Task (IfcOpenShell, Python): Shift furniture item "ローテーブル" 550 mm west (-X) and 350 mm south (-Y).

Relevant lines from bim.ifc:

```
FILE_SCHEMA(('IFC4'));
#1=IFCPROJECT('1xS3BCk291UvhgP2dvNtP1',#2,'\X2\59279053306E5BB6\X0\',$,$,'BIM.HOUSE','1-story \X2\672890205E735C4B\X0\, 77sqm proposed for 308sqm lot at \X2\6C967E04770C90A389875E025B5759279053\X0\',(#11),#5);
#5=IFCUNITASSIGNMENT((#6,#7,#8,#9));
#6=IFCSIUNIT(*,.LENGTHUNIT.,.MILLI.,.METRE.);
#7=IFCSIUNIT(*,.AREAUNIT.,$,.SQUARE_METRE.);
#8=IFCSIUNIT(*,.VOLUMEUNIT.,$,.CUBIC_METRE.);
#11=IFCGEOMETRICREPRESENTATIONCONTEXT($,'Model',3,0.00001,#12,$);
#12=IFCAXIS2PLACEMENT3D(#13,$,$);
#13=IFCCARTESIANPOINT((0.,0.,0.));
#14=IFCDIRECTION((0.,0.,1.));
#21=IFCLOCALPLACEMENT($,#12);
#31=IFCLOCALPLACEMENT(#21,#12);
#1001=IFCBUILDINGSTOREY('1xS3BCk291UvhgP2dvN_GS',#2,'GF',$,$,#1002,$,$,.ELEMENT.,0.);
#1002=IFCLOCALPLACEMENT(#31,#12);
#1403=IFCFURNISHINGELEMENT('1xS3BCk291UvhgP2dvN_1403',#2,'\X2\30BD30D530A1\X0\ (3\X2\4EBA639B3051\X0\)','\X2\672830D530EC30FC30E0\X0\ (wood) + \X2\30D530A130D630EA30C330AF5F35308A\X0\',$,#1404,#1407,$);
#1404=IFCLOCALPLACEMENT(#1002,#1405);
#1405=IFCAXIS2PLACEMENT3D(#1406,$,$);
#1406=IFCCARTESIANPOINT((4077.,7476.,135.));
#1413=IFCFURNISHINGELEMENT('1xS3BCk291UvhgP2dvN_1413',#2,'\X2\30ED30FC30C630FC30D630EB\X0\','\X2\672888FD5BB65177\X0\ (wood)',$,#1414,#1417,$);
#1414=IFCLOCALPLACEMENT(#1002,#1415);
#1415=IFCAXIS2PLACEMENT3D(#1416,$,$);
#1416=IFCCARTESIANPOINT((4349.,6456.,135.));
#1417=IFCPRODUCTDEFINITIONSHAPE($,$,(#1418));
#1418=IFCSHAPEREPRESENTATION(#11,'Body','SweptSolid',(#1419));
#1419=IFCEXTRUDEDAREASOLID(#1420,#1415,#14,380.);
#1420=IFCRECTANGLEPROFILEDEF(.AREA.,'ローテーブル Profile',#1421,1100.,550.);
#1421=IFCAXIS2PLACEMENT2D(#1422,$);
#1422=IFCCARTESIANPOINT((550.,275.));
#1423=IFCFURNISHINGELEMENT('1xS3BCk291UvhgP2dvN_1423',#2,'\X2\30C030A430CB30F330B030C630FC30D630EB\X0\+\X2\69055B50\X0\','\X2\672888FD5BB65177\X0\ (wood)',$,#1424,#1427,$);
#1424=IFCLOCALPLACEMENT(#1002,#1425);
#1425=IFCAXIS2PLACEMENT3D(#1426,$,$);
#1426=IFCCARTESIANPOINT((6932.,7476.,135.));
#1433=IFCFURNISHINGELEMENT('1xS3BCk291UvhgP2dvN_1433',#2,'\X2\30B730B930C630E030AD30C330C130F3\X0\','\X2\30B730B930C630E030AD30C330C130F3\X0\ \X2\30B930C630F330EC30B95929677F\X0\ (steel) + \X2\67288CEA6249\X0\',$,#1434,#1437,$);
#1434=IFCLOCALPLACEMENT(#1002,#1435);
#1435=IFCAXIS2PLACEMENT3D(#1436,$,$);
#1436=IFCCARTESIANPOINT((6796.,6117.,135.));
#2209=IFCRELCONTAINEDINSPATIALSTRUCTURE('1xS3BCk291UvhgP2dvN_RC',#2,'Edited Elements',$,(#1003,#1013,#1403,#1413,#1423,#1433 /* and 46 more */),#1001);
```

```python
import ifcopenshell
import ifcopenshell.api.geometry
import ifcopenshell.util.placement

model = ifcopenshell.open("bim.ifc")

item = model.by_id(1413)
matrix = ifcopenshell.util.placement.get_local_placement(item.ObjectPlacement)
matrix[0, 3] -= 550.0
matrix[1, 3] -= 350.0
ifcopenshell.api.geometry.edit_object_placement(model, product=item, matrix=matrix, is_si=False)

print(ifcopenshell.util.placement.get_local_placement(item.ObjectPlacement).round(3) + 0.0)

model.write("bim-out.ifc")
```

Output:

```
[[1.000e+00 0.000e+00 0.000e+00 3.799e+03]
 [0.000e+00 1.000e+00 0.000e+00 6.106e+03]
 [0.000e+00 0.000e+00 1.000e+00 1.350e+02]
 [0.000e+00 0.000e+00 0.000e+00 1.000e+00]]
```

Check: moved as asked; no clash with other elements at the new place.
